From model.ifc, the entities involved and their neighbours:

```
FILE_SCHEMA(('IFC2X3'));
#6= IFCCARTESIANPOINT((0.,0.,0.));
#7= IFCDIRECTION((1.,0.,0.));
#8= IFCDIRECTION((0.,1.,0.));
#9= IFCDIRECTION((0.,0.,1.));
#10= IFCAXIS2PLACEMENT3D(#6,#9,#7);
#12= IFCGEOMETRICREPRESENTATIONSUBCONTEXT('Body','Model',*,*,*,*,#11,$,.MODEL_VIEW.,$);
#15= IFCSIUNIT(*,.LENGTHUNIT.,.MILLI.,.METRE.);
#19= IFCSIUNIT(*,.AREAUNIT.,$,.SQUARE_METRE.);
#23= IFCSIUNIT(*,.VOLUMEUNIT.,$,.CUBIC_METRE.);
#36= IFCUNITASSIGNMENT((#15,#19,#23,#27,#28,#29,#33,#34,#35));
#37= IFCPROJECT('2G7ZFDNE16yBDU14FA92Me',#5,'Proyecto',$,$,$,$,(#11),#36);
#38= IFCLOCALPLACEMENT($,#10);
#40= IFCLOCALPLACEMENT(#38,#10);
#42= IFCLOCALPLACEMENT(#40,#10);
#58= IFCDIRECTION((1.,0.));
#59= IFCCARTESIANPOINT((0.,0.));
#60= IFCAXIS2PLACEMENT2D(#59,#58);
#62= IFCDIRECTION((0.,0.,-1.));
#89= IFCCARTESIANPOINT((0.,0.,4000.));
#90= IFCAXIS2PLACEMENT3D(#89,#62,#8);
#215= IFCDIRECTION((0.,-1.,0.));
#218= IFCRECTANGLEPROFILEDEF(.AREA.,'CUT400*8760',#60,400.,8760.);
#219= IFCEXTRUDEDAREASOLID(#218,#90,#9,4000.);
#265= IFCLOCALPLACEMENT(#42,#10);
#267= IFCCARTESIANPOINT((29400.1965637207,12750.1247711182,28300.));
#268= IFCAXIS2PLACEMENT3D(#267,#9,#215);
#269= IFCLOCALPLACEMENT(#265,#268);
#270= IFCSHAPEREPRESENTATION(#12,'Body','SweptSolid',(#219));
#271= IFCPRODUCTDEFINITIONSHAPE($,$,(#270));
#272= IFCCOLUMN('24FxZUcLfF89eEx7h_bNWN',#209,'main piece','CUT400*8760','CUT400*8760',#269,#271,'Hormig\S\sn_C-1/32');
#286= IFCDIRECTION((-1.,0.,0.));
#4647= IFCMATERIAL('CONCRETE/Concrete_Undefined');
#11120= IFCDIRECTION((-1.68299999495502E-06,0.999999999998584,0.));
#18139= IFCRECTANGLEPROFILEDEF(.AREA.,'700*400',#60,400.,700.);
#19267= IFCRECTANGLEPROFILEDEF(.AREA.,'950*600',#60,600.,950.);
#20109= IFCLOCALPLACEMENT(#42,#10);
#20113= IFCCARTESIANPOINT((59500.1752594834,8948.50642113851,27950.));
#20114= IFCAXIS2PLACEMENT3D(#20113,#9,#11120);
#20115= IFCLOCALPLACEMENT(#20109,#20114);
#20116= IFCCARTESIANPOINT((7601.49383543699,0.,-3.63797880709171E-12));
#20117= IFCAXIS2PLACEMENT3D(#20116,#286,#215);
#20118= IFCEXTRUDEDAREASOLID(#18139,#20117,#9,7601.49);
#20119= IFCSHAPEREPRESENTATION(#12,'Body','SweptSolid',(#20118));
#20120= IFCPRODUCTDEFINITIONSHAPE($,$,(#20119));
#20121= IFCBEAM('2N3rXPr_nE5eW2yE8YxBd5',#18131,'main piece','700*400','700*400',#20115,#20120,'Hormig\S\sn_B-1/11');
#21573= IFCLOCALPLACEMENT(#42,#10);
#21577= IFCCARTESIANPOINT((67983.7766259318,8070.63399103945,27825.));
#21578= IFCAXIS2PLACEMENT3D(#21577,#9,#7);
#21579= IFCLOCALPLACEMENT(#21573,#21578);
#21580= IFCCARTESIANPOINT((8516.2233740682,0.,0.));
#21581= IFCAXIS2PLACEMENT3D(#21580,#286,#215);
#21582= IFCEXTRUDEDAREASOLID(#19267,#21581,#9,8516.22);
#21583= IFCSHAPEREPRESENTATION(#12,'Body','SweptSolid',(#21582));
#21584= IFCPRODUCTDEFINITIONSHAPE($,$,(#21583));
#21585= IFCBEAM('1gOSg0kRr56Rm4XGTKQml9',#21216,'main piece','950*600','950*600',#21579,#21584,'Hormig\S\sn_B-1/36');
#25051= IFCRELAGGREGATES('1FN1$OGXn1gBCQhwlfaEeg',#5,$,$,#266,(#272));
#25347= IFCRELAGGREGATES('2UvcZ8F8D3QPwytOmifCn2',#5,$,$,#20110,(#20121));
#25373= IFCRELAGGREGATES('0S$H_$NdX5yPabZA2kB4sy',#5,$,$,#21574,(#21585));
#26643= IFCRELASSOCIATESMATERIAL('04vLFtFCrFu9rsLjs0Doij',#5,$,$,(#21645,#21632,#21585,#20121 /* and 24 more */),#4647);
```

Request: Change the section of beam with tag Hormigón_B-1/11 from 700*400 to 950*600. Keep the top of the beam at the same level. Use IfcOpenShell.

```python
import ifcopenshell
import ifcopenshell.util.element
import ifcopenshell.util.representation

model = ifcopenshell.open("model.ifc")

member = model.by_id(20121)
source = next(p for p in model.by_type("IfcRectangleProfileDef") if p.ProfileName == "950*600")

body = ifcopenshell.util.representation.get_representation(member, "Model", "Body")
solid = body.Items[0]
old_profile = solid.SweptArea

# Copy the section's sizes but keep this member's own profile position.
profile = ifcopenshell.util.element.copy(model, source)
# Profiles are centred, so shift by half the change in depth to hold the top.
shift = (old_profile.YDim - profile.YDim) / 2
x, y = old_profile.Position.Location.Coordinates
up = (0.0, 1.0)  # upwards, in the solid's own plane
location = model.createIfcCartesianPoint((x + up[0] * shift, y + up[1] * shift))
profile.Position = model.createIfcAxis2Placement2D(location, old_profile.Position.RefDirection)
solid.SweptArea = profile
if not model.get_total_inverses(old_profile):
    ifcopenshell.util.element.remove_deep2(model, old_profile)
member.Description = member.Description.replace("700*400", "950*600")
member.ObjectType = member.ObjectType.replace("700*400", "950*600")

print(solid.SweptArea)

model.write("model_updated.ifc")
```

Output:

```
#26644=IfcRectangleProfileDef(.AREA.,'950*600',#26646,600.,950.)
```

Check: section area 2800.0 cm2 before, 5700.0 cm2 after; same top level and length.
